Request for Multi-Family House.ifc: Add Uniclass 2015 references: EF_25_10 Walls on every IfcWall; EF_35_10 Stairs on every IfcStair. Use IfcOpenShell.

First a look at what the model holds.

```python
import ifcopenshell

model = ifcopenshell.open("Multi-Family House.ifc")
print(model.schema)
print("classifications:", [c.Name for c in model.by_type("IfcClassification")])
for ifc_class in ("IfcDoor", "IfcRoof", "IfcStair", "IfcWall", "IfcWindow"):
    print(ifc_class, len(model.by_type(ifc_class)))
```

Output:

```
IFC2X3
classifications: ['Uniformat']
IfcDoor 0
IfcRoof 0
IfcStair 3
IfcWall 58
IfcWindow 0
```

```python
import ifcopenshell
import ifcopenshell.api.classification

model = ifcopenshell.open("Multi-Family House.ifc")

# IFC2X3 requires Source and Edition and has no link from the project to the system.
system = model.create_entity("IfcClassification", Source="NBS", Edition="2015", Name="Uniclass 2015")

codes = {
    "IfcWall": ("EF_25_10", "Walls"),
    "IfcStair": ("EF_35_10", "Stairs"),
}
for ifc_class, (code, name) in codes.items():
    products = model.by_type(ifc_class)
    ifcopenshell.api.classification.add_reference(
        model, products=products, classification=system, identification=code, name=name
    )
    print(code, len(products))

model.write("Multi-Family House_rev.ifc")
```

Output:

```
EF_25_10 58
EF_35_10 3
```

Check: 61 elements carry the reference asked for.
